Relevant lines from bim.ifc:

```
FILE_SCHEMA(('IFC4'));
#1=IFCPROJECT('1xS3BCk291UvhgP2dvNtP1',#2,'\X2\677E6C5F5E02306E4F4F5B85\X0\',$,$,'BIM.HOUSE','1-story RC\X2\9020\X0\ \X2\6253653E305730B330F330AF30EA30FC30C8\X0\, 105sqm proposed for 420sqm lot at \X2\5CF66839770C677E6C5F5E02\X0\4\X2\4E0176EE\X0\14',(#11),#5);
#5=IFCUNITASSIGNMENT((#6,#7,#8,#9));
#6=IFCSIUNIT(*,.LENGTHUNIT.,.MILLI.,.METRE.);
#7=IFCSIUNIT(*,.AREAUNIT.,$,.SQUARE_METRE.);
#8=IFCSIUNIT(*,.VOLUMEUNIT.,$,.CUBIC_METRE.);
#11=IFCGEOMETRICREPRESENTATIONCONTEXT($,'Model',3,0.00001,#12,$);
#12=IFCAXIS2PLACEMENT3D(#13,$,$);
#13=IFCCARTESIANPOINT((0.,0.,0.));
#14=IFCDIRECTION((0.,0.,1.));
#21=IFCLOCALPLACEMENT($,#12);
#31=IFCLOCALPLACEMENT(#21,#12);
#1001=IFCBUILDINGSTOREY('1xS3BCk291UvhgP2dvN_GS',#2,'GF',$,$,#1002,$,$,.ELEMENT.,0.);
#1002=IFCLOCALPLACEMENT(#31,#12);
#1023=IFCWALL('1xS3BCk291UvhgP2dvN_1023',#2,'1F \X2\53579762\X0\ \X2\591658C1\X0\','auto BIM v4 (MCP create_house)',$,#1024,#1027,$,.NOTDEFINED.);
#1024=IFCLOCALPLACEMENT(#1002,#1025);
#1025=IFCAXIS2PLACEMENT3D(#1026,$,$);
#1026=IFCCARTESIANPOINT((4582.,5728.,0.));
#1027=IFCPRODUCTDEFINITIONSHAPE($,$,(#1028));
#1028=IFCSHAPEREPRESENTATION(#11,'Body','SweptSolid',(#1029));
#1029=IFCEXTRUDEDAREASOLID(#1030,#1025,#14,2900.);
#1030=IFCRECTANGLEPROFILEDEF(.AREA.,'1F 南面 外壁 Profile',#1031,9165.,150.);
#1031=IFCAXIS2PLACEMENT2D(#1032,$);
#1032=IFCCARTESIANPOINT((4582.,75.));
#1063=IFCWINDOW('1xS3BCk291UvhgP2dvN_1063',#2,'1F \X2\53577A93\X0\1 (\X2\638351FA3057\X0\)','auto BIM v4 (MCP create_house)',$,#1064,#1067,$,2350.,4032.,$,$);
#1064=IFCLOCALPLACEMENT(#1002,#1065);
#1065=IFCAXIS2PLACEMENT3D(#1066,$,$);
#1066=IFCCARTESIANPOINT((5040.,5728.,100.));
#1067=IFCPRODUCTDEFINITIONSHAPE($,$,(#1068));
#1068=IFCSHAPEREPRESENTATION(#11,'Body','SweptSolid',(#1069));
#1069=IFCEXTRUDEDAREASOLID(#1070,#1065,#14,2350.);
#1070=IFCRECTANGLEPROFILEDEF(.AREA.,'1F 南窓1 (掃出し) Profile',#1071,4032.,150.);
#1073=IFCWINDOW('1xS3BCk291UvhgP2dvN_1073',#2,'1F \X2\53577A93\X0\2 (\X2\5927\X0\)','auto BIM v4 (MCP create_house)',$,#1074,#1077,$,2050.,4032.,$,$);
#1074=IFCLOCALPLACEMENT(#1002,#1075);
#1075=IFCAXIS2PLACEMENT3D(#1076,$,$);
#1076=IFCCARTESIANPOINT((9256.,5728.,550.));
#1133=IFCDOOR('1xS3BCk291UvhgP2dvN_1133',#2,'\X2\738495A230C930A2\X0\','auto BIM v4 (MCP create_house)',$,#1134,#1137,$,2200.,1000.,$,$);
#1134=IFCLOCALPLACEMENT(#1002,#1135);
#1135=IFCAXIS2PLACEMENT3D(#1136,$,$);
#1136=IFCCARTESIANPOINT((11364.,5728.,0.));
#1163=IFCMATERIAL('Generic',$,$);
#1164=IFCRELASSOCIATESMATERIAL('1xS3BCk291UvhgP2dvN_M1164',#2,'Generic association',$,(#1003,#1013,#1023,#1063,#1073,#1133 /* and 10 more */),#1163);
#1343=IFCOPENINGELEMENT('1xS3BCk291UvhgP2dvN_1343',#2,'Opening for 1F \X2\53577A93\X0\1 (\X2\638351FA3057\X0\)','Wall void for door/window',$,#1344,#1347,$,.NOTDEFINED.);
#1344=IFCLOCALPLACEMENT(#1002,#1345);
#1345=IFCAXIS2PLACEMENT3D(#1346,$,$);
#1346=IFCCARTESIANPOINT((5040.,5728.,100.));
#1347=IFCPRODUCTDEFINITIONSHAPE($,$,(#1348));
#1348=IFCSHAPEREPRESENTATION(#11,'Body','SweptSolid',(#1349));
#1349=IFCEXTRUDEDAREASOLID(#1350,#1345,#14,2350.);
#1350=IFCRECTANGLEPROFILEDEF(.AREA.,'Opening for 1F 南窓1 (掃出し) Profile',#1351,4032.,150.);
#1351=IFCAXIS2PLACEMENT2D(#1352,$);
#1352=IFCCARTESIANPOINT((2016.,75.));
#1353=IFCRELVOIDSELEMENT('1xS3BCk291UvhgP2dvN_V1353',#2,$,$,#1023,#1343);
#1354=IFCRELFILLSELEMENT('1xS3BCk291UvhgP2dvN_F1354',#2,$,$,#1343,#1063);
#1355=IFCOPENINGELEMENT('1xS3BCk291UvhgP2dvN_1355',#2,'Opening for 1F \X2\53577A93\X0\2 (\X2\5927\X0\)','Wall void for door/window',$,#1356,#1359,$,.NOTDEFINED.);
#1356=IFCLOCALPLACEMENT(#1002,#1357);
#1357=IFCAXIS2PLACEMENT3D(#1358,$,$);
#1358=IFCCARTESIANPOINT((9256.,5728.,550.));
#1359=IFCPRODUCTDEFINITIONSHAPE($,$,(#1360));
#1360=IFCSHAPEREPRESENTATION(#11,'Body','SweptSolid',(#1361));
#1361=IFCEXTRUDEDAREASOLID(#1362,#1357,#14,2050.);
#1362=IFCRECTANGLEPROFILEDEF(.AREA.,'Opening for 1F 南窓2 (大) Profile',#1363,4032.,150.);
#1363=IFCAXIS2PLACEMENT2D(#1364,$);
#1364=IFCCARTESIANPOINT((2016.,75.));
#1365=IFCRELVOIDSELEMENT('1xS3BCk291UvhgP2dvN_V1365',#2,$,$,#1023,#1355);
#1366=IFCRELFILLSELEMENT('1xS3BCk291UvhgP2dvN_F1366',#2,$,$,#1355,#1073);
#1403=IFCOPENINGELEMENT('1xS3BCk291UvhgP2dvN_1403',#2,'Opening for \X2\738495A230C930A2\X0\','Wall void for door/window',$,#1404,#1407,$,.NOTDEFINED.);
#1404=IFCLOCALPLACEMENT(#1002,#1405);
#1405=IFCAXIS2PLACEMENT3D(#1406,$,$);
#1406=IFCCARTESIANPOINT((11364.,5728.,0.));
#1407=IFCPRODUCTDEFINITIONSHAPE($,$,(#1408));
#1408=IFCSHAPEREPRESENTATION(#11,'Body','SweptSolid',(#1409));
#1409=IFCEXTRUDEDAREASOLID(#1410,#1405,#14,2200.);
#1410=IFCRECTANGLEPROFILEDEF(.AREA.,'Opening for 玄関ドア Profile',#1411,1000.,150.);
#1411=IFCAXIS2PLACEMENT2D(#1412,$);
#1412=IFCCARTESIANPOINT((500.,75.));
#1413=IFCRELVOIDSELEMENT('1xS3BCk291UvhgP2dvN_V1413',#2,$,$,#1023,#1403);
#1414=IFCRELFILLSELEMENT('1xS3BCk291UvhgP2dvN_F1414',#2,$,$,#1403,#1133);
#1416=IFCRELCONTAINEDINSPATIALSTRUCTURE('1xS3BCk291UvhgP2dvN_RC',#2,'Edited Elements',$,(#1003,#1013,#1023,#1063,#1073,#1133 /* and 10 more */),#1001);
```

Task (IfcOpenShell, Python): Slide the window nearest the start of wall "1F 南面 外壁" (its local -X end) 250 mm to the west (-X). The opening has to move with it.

```python
import ifcopenshell
import ifcopenshell.api.geometry
import ifcopenshell.util.placement
import ifcopenshell.util.unit

model = ifcopenshell.open("bim.ifc")
unit_scale = ifcopenshell.util.unit.calculate_unit_scale(model)

window = model.by_guid("1xS3BCk291UvhgP2dvN_1063")
opening = window.FillsVoids[0].RelatingOpeningElement
wall = opening.VoidsElements[0].RelatingBuildingElement

wall_matrix = ifcopenshell.util.placement.get_local_placement(wall.ObjectPlacement)
shift = wall_matrix[:3, 0] * -0.25 / unit_scale
before = ifcopenshell.util.placement.get_local_placement(window.ObjectPlacement)[:3, 3].copy()

# The window is not placed relative to its opening, so move both.
for product in (opening, window):
    matrix = ifcopenshell.util.placement.get_local_placement(product.ObjectPlacement)
    matrix[:3, 3] += shift
    ifcopenshell.api.geometry.edit_object_placement(model, product=product, matrix=matrix, is_si=False)

after = ifcopenshell.util.placement.get_local_placement(window.ObjectPlacement)[:3, 3]
print("window moved by", (after - before).round(3) + 0.0)

model.write("bim_updated.ifc")
```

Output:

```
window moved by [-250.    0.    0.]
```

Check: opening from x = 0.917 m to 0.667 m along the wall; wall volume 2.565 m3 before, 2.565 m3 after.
